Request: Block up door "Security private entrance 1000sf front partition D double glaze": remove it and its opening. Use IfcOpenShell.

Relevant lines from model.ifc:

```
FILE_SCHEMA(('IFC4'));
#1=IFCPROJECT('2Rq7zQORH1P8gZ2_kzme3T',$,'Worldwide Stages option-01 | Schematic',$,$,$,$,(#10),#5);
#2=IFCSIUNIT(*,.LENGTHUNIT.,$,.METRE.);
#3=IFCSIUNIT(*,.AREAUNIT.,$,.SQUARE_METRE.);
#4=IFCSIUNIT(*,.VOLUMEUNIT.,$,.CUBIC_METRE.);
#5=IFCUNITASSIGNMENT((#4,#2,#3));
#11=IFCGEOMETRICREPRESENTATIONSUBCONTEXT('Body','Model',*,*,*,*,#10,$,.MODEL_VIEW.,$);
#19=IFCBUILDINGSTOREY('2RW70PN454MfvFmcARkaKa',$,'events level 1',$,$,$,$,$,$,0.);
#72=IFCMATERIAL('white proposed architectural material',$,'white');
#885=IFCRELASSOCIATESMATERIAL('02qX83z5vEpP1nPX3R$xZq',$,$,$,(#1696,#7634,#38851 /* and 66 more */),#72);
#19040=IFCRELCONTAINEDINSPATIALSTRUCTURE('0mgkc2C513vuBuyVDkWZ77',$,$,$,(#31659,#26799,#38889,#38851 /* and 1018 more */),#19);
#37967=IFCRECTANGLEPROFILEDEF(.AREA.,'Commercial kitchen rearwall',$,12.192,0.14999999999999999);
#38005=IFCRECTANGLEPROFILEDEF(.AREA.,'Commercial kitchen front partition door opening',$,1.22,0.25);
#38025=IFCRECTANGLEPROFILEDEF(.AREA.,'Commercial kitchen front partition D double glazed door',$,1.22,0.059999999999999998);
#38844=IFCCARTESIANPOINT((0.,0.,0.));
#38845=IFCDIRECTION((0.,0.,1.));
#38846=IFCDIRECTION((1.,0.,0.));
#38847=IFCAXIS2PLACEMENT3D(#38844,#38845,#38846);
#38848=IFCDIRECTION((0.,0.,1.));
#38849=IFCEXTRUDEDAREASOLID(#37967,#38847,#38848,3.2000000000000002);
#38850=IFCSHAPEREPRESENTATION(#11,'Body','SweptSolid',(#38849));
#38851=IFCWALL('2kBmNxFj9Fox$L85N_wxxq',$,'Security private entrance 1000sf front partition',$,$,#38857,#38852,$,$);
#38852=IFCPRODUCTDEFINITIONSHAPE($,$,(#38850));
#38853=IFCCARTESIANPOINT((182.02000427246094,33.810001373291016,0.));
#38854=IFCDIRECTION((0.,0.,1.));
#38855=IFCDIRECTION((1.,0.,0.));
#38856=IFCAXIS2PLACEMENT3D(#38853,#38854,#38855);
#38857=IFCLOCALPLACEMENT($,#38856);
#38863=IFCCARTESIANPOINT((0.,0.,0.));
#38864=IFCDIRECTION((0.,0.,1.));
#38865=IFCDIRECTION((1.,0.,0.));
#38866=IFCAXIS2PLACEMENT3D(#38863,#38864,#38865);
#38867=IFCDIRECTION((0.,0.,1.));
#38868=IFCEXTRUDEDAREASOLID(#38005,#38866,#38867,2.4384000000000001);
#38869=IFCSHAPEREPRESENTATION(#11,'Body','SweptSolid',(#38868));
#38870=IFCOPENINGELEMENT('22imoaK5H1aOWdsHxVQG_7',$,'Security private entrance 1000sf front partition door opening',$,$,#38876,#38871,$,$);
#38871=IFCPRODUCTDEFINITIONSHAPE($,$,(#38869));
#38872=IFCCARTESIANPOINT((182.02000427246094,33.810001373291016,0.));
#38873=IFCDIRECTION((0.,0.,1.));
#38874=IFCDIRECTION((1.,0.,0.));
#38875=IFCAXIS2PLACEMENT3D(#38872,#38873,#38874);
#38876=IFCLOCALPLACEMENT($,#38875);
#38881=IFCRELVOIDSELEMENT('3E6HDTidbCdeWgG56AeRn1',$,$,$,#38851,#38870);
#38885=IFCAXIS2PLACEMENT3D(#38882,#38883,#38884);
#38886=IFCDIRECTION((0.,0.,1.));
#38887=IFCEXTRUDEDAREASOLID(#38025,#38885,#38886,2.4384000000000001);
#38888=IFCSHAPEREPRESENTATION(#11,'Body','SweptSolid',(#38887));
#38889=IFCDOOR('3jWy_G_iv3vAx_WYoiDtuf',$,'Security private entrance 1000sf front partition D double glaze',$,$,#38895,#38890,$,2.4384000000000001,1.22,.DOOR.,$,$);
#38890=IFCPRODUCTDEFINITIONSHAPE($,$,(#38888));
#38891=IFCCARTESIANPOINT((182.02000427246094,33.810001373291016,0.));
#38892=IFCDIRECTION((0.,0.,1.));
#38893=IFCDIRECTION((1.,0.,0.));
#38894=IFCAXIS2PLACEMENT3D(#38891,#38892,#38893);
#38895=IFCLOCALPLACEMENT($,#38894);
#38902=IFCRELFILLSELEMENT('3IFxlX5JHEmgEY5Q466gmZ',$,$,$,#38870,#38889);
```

```python
import ifcopenshell
import ifcopenshell.api.feature
import ifcopenshell.api.root
import ifcopenshell.geom
import ifcopenshell.util.shape

model = ifcopenshell.open("model.ifc")
settings = ifcopenshell.geom.settings()


def volume(element):
    """Net volume in cubic metres, openings subtracted."""
    shape = ifcopenshell.geom.create_shape(settings, element)
    return ifcopenshell.util.shape.get_volume(shape.geometry)


door = model.by_guid("3jWy_G_iv3vAx_WYoiDtuf")
opening = door.FillsVoids[0].RelatingOpeningElement
wall = opening.VoidsElements[0].RelatingBuildingElement
before = volume(wall)

ifcopenshell.api.root.remove_product(model, product=door)
ifcopenshell.api.feature.remove_feature(model, feature=opening)

after = volume(wall)

print(f"wall volume {before:.3f} -> {after:.3f} m3")

model.write("model_rev.ifc")
```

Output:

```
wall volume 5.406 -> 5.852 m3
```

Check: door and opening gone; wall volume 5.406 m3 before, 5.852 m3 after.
